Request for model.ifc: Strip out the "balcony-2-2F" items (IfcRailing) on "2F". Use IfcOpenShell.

First a look at what the model holds.

```python
import ifcopenshell
import ifcopenshell.util.element

model = ifcopenshell.open("model.ifc")
print(model.schema)
storey = next(s for s in model.by_type("IfcBuildingStorey") if s.Name == "2F")
railings = [e for e in ifcopenshell.util.element.get_decomposition(storey) if e.is_a("IfcRailing")]
seen = {}
for e in railings:
    element_type = ifcopenshell.util.element.get_type(e)
    name = element_type.Name if element_type not in (None, e) else None
    seen[name] = seen.get(name, 0) + 1
for name, count in sorted(seen.items(), key=str):
    print(count, "x", name)
```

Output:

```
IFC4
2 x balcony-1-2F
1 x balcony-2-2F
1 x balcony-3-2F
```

```python
import ifcopenshell
import ifcopenshell.api.root
import ifcopenshell.util.element

model = ifcopenshell.open("model.ifc")

storey = next(s for s in model.by_type("IfcBuildingStorey") if s.Name == "2F")
railings = [e for e in ifcopenshell.util.element.get_decomposition(storey) if e.is_a("IfcRailing")]
targets = [e for e in railings if (t := ifcopenshell.util.element.get_type(e)) not in (None, e) and t.Name == "balcony-2-2F"]

for e in targets:
    ifcopenshell.api.root.remove_product(model, product=e)
print(len(targets), "removed")

model.write("model_updated.ifc")
```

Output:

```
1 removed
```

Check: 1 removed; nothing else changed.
